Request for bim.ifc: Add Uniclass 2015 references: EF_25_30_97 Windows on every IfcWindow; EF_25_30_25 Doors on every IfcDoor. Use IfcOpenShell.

First a look at what the model holds.

```python
import ifcopenshell

model = ifcopenshell.open("bim.ifc")
print(model.schema)
print("classifications:", [c.Name for c in model.by_type("IfcClassification")])
for ifc_class in ("IfcDoor", "IfcRoof", "IfcStair", "IfcWall", "IfcWindow"):
    print(ifc_class, len(model.by_type(ifc_class)))
```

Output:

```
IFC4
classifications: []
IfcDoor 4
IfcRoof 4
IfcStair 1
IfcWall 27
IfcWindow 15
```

```python
import ifcopenshell
import ifcopenshell.api.classification

model = ifcopenshell.open("bim.ifc")

system = ifcopenshell.api.classification.add_classification(model, classification="Uniclass 2015")

codes = {
    "IfcWindow": ("EF_25_30_97", "Windows"),
    "IfcDoor": ("EF_25_30_25", "Doors"),
}
for ifc_class, (code, name) in codes.items():
    products = model.by_type(ifc_class)
    ifcopenshell.api.classification.add_reference(
        model, products=products, classification=system, identification=code, name=name
    )
    print(code, len(products))

model.write("bim_v2.ifc")
```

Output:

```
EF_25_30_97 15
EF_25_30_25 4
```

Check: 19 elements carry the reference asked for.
